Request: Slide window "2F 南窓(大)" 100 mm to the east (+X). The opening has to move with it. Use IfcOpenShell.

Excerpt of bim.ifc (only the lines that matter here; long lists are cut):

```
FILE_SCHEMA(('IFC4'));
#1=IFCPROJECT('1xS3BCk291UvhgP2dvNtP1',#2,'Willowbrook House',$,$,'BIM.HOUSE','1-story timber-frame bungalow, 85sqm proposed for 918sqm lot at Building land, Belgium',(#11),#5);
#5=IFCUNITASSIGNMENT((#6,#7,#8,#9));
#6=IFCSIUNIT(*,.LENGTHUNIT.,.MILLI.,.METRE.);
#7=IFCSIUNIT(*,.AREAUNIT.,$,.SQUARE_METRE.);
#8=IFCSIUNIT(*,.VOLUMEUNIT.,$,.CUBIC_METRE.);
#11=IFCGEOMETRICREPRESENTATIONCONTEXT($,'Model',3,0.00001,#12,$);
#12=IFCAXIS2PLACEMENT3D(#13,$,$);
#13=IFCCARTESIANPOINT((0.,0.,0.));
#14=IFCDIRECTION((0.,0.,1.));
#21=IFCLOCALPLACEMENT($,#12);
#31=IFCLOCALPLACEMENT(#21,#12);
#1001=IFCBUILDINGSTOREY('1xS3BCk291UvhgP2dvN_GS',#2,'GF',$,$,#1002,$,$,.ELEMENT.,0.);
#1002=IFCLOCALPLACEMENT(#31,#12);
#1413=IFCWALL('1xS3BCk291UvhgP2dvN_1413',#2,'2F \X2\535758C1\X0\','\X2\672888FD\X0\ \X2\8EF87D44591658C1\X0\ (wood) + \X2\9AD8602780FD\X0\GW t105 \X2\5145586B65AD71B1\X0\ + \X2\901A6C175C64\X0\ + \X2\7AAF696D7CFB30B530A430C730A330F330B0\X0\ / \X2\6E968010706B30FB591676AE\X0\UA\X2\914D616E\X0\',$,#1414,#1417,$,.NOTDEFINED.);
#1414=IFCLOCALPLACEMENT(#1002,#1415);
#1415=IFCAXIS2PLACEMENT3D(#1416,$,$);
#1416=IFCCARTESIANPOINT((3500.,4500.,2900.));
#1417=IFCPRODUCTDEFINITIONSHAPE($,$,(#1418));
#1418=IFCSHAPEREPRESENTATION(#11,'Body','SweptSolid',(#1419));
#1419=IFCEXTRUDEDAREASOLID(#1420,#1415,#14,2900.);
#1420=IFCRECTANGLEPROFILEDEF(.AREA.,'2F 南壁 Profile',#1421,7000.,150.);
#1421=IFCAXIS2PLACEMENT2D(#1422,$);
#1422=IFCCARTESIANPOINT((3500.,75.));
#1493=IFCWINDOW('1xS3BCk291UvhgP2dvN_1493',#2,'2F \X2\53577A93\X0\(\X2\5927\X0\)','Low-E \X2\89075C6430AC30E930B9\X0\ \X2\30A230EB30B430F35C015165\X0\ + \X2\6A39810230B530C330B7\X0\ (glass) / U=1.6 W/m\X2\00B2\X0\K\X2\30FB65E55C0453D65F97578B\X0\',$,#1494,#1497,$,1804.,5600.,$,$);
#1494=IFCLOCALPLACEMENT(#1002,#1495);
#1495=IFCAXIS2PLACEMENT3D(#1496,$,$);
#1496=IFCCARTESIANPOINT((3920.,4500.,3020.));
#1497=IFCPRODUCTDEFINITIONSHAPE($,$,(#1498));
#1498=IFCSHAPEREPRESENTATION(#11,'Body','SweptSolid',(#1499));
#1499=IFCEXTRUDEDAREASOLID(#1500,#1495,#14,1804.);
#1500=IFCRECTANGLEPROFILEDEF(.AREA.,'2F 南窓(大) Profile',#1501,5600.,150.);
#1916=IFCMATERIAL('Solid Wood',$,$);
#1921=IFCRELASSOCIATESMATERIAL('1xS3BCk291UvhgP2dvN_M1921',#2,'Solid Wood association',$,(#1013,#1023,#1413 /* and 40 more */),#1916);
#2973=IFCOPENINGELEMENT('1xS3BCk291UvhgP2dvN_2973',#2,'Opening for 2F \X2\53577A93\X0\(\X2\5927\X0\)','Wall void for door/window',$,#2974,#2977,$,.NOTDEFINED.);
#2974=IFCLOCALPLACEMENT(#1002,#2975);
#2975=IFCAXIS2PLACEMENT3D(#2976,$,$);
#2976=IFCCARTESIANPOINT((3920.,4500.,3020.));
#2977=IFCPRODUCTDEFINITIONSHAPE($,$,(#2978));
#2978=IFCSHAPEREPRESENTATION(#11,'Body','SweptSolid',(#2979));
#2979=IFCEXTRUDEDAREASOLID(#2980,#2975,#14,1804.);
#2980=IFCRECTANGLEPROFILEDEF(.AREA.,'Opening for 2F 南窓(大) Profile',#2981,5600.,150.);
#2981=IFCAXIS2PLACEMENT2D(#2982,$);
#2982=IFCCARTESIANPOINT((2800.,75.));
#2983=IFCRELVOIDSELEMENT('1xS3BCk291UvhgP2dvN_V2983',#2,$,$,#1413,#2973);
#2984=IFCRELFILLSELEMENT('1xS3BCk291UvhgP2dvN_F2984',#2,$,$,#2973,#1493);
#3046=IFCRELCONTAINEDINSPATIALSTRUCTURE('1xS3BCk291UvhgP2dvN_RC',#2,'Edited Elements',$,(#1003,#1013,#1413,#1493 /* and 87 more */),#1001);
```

```python
import ifcopenshell
import ifcopenshell.api.geometry
import ifcopenshell.util.placement
import ifcopenshell.util.unit

model = ifcopenshell.open("bim.ifc")
unit_scale = ifcopenshell.util.unit.calculate_unit_scale(model)

window = model.by_id(1493)
opening = window.FillsVoids[0].RelatingOpeningElement
wall = opening.VoidsElements[0].RelatingBuildingElement

wall_matrix = ifcopenshell.util.placement.get_local_placement(wall.ObjectPlacement)
shift = wall_matrix[:3, 0] * 0.1 / unit_scale
before = ifcopenshell.util.placement.get_local_placement(window.ObjectPlacement)[:3, 3].copy()

# The window is not placed relative to its opening, so move both.
for product in (opening, window):
    matrix = ifcopenshell.util.placement.get_local_placement(product.ObjectPlacement)
    matrix[:3, 3] += shift
    ifcopenshell.api.geometry.edit_object_placement(model, product=product, matrix=matrix, is_si=False)

after = ifcopenshell.util.placement.get_local_placement(window.ObjectPlacement)[:3, 3]
print("window moved by", (after - before).round(3) + 0.0)

model.write("bim_updated.ifc")
```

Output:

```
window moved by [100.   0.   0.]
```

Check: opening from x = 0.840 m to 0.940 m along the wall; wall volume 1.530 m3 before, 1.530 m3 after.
